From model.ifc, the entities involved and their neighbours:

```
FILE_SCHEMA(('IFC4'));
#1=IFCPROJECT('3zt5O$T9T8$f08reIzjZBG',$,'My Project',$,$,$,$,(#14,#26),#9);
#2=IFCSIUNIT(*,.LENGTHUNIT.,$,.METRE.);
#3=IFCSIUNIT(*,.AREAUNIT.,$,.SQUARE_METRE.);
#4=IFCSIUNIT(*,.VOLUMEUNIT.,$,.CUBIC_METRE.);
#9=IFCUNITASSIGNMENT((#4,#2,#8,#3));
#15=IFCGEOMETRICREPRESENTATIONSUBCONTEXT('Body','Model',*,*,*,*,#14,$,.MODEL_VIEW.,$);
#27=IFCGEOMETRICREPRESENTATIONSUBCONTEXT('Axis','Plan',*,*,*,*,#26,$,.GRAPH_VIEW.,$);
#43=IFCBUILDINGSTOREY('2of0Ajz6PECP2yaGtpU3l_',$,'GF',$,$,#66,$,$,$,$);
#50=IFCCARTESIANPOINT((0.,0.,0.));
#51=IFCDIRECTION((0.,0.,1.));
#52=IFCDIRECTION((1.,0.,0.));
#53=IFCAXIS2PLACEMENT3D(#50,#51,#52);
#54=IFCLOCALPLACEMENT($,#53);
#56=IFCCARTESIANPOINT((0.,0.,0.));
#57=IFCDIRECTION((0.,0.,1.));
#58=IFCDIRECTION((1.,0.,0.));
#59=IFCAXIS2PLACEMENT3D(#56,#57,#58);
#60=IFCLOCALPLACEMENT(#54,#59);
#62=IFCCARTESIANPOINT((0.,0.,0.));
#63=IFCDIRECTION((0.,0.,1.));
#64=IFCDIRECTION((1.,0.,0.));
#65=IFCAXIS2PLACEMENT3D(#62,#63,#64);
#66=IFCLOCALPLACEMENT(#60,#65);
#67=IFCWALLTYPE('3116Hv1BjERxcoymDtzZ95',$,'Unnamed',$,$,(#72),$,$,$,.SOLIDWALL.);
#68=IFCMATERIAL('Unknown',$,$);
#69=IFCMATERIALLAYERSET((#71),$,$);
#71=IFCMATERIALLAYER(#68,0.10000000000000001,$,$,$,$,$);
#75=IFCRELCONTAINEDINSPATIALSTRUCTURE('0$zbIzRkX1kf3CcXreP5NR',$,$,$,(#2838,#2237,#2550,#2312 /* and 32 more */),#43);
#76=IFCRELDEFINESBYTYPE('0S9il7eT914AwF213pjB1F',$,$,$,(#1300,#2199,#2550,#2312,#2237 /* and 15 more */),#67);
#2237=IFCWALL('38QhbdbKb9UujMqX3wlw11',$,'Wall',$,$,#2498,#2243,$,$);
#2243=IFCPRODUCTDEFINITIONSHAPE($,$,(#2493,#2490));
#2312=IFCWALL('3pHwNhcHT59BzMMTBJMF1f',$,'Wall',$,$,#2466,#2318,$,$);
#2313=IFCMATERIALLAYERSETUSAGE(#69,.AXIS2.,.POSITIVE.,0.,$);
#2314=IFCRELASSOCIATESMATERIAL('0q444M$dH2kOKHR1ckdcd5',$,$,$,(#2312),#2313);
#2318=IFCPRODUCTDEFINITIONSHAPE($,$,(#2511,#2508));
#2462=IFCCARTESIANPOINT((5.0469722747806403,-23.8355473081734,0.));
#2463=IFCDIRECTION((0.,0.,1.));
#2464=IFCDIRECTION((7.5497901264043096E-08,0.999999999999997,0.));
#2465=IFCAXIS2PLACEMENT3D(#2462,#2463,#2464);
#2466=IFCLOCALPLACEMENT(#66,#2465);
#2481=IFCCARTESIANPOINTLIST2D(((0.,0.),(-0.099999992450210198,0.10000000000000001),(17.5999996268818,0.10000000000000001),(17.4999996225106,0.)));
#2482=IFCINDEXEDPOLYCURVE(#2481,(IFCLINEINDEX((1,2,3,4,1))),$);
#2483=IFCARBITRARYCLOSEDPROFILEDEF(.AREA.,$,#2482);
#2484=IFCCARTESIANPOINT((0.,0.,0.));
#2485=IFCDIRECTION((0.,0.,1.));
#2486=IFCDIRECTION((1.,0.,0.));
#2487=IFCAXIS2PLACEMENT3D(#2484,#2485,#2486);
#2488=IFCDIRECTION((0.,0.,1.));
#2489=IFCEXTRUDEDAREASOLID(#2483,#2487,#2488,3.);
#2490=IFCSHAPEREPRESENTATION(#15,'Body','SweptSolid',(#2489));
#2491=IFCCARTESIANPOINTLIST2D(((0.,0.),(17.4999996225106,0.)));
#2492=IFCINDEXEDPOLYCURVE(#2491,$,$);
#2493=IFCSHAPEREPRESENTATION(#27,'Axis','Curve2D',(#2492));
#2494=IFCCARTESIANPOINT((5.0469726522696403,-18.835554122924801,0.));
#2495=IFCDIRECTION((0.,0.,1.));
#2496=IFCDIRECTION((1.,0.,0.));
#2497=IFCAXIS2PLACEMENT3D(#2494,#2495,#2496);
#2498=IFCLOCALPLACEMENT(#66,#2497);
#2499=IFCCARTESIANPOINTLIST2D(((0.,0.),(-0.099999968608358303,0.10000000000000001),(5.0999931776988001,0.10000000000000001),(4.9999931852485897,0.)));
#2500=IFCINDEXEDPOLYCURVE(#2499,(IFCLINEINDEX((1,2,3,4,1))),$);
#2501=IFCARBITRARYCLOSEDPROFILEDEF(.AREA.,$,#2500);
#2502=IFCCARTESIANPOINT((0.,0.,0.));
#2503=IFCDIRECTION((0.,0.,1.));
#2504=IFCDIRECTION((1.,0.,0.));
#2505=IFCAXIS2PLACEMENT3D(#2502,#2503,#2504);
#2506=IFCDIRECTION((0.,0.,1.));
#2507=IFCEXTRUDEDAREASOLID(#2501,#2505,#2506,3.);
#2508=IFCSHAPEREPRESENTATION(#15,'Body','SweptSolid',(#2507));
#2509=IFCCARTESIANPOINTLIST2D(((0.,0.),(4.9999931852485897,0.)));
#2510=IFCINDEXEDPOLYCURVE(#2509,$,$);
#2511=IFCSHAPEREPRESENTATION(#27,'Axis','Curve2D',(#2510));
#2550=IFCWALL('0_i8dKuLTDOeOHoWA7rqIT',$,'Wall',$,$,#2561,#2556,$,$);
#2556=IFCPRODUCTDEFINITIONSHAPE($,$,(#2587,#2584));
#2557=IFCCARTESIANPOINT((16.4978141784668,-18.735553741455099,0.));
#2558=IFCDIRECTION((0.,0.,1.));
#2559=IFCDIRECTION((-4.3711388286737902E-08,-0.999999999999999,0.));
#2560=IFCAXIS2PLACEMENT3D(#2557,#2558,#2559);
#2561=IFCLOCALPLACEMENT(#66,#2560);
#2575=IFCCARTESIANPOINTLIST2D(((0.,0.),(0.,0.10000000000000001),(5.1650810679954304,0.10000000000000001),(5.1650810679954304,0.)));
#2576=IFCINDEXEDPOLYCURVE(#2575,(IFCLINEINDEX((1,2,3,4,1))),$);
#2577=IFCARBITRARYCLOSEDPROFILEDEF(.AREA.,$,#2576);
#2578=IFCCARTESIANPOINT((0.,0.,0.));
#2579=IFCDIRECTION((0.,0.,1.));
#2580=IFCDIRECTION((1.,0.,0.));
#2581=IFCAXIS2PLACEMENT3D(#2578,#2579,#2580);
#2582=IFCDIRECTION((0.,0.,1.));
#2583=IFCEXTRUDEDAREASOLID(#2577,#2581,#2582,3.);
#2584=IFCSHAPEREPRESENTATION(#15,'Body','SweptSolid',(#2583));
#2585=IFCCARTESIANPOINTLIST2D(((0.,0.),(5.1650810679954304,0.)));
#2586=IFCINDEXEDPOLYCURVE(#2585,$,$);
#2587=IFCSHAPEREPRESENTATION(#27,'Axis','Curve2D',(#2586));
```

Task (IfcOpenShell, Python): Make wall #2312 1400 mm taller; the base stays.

```python
import ifcopenshell
import ifcopenshell.geom
import ifcopenshell.util.representation
import ifcopenshell.util.shape
import ifcopenshell.util.unit

model = ifcopenshell.open("model.ifc")
unit_scale = ifcopenshell.util.unit.calculate_unit_scale(model)
settings = ifcopenshell.geom.settings()


def volume(element):
    """Net volume in cubic metres, openings subtracted."""
    shape = ifcopenshell.geom.create_shape(settings, element)
    return ifcopenshell.util.shape.get_volume(shape.geometry)


wall = model.by_id(2312)
before = volume(wall)

body = ifcopenshell.util.representation.get_representation(wall, "Model", "Body")
solid = body.Items[0]
old_height = solid.Depth
solid.Depth += 1.4 / unit_scale
after = volume(wall)

print(f"height {old_height:g} -> {solid.Depth:g}, volume {before:.3f} -> {after:.3f} m3")

model.write("model_v2.ifc")
```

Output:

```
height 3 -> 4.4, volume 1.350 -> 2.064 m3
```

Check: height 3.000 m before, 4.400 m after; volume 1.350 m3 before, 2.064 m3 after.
